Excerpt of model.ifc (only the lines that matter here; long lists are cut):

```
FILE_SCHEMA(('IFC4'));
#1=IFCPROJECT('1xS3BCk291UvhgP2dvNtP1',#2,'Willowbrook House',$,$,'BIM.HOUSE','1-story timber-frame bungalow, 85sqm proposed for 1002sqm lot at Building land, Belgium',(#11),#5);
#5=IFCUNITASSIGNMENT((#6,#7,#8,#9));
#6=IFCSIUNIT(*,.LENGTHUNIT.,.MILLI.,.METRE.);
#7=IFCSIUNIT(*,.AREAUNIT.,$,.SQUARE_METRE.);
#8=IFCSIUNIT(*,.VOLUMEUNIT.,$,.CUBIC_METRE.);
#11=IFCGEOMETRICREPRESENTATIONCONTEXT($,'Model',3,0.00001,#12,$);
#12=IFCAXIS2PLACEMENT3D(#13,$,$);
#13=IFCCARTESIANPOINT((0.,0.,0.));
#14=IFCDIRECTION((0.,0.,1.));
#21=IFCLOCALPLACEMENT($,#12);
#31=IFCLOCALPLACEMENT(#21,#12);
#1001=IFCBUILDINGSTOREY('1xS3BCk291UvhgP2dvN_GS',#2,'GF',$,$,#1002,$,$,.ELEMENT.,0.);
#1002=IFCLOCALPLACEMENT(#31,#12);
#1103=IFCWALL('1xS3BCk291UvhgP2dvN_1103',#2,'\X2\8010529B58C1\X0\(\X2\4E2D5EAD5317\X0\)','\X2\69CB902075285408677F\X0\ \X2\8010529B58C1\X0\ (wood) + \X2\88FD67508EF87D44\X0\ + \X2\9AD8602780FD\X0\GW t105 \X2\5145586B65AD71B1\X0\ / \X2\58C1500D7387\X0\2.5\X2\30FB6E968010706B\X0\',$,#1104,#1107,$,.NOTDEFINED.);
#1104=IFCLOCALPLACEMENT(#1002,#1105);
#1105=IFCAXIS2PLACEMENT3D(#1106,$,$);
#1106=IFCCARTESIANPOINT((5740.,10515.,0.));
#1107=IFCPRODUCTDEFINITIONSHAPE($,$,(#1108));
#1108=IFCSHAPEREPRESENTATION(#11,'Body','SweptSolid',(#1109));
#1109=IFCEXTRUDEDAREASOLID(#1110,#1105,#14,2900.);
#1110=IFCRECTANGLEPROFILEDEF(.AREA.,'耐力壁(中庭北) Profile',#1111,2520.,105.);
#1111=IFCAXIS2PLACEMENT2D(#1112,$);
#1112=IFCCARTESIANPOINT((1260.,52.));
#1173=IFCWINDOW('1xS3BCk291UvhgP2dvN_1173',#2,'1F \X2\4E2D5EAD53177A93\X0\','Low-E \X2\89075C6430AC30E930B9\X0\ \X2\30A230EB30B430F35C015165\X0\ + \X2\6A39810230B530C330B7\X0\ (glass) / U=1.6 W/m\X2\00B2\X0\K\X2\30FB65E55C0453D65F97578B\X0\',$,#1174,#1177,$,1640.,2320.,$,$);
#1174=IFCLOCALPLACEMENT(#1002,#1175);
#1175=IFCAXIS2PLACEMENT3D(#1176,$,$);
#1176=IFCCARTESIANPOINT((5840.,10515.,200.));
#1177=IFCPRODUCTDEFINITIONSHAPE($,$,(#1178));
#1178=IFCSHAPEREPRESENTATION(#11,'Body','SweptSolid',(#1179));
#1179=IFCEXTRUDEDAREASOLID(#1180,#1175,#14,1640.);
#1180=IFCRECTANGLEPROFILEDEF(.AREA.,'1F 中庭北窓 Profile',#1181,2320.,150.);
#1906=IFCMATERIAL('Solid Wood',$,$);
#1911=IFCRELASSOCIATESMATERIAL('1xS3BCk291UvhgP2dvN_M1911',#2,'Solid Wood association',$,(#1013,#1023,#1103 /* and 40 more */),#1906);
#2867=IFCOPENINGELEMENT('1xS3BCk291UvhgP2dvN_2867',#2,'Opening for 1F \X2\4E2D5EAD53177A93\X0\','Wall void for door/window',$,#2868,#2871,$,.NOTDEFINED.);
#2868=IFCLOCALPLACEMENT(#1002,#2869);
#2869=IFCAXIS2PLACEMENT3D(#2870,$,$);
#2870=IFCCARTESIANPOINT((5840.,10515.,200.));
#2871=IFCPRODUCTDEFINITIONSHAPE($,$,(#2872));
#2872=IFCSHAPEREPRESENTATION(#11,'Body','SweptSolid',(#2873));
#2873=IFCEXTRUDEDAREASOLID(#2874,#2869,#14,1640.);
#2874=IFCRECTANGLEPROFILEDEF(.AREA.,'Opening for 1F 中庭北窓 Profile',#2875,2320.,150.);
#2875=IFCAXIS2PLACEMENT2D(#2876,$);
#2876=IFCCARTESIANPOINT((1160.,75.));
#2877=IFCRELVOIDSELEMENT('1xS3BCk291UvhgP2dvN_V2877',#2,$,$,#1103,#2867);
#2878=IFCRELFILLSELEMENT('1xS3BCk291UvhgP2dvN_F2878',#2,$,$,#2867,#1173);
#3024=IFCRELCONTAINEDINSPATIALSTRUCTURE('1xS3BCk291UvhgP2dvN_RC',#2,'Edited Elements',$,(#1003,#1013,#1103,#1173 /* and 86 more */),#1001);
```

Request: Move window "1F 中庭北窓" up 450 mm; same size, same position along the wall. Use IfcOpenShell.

```python
import numpy as np
import ifcopenshell
import ifcopenshell.api.geometry
import ifcopenshell.util.placement
import ifcopenshell.util.unit

model = ifcopenshell.open("model.ifc")
unit_scale = ifcopenshell.util.unit.calculate_unit_scale(model)

window = model.by_guid("1xS3BCk291UvhgP2dvN_1173")
opening = window.FillsVoids[0].RelatingOpeningElement
dz = 450.0

shift = np.array([0.0, 0.0, dz])
# The window is not placed relative to its opening, so move both.
for product in (opening, window):
    matrix = ifcopenshell.util.placement.get_local_placement(product.ObjectPlacement)
    matrix[:3, 3] += shift
    ifcopenshell.api.geometry.edit_object_placement(model, product=product, matrix=matrix, is_si=False)

print(f"moved by {dz * unit_scale:+.3f} m")

model.write("model_v2.ifc")
```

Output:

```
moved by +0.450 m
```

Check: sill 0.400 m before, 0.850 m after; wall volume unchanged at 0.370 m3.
